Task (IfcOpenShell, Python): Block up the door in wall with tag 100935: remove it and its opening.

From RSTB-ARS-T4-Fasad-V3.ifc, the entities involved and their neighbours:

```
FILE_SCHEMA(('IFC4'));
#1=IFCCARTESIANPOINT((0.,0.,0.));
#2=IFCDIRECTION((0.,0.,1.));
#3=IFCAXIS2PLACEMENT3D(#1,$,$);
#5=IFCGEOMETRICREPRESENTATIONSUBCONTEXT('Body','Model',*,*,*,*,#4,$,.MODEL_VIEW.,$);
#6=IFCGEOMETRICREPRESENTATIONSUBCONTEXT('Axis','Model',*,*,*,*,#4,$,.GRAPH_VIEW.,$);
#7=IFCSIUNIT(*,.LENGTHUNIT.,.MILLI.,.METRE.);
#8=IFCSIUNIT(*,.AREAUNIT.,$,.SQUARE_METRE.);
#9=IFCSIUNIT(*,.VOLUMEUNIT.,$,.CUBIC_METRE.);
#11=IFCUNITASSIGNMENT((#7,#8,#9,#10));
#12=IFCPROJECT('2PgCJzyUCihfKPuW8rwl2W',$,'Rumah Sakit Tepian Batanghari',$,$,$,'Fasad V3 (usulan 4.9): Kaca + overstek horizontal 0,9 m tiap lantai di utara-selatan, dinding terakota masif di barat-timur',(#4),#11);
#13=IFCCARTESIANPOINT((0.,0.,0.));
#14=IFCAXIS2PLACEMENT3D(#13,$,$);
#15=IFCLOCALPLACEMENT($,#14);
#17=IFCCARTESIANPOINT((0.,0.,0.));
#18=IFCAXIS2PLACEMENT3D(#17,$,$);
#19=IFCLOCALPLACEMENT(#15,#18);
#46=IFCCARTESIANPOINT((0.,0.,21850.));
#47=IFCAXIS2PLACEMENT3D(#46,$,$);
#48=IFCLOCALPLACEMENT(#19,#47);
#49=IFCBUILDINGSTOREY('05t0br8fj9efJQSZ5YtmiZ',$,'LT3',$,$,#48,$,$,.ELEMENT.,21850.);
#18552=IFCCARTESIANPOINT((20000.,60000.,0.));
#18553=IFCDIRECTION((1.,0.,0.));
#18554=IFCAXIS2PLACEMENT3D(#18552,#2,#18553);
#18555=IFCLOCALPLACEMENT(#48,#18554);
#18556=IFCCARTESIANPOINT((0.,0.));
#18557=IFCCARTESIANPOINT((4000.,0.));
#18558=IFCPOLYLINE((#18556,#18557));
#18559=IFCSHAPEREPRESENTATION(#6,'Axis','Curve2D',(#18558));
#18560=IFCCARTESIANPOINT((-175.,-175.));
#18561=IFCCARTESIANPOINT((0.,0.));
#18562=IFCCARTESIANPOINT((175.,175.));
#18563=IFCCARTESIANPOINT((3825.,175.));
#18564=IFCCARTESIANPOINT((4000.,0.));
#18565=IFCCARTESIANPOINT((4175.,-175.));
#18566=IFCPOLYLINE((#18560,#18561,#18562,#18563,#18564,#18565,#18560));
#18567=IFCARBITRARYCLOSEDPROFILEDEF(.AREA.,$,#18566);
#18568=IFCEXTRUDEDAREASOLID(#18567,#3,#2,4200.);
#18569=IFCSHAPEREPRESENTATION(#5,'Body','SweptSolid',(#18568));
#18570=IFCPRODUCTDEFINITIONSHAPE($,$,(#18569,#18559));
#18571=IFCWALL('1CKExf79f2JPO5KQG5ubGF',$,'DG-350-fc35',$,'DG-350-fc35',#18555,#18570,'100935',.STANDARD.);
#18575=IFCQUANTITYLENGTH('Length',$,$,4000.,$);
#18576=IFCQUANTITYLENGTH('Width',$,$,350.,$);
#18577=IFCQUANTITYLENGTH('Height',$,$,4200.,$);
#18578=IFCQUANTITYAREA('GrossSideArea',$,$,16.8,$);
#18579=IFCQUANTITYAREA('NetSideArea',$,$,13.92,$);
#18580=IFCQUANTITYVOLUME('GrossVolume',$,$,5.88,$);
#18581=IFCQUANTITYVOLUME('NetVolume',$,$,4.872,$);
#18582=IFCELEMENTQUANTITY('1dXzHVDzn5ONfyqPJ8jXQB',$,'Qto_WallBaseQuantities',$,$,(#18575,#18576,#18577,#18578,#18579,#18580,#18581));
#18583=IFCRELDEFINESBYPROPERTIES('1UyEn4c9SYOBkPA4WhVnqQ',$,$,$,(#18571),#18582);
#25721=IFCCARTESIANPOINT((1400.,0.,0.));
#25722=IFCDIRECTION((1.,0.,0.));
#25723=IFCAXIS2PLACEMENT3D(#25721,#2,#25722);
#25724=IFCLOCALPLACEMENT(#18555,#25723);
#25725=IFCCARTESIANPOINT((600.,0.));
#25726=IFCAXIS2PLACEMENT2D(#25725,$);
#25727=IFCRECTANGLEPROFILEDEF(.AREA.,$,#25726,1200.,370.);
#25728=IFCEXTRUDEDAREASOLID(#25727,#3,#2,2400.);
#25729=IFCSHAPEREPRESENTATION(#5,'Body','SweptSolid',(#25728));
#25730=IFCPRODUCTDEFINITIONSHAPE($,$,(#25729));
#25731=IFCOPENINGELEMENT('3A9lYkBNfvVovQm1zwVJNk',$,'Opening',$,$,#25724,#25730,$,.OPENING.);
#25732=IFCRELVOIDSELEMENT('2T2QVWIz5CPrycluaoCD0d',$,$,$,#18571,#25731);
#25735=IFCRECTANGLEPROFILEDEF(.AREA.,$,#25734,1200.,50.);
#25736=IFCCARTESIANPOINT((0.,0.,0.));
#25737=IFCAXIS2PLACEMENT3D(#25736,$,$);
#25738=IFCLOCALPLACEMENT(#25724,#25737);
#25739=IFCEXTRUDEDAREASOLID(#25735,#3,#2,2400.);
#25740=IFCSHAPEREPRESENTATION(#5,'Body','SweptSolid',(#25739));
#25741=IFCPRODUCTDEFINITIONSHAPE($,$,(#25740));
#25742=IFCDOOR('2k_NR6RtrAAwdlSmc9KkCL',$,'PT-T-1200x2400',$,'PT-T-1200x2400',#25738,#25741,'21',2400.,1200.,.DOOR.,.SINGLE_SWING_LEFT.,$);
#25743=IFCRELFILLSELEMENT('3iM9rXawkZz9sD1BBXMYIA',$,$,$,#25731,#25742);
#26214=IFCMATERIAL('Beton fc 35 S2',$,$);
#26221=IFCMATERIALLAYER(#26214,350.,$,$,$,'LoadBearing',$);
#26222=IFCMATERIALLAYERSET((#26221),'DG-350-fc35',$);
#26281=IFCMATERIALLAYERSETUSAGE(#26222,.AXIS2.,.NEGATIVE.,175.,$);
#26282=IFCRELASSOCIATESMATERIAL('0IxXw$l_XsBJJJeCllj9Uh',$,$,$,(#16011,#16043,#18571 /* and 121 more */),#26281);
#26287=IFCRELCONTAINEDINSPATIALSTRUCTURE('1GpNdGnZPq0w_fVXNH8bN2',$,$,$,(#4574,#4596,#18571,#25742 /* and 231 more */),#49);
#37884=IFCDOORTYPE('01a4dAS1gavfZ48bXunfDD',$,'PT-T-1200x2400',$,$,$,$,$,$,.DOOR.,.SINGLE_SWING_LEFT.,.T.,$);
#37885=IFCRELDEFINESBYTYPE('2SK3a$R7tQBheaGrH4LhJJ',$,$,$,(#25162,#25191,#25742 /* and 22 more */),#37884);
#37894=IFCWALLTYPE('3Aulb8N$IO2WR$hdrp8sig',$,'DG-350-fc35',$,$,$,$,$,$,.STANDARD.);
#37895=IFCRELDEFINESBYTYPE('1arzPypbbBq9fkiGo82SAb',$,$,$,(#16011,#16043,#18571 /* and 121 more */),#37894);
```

```python
import ifcopenshell
import ifcopenshell.api.feature
import ifcopenshell.api.pset
import ifcopenshell.api.root
import ifcopenshell.geom
import ifcopenshell.util.element
import ifcopenshell.util.shape
import ifcopenshell.util.unit

model = ifcopenshell.open("RSTB-ARS-T4-Fasad-V3.ifc")
area_scale = ifcopenshell.util.unit.calculate_unit_scale(model, "AREAUNIT")
volume_scale = ifcopenshell.util.unit.calculate_unit_scale(model, "VOLUMEUNIT")
settings = ifcopenshell.geom.settings()


def volume(element):
    """Net volume in cubic metres, openings subtracted."""
    shape = ifcopenshell.geom.create_shape(settings, element)
    return ifcopenshell.util.shape.get_volume(shape.geometry)


door = model.by_id(25742)
opening = door.FillsVoids[0].RelatingOpeningElement
wall = opening.VoidsElements[0].RelatingBuildingElement
before = volume(wall)

ifcopenshell.api.root.remove_product(model, product=door)
ifcopenshell.api.feature.remove_feature(model, feature=opening)

after = volume(wall)
thickness = 0.35  # wall thickness in metres

# Update the wall's stored quantities.
qto = model.by_id(ifcopenshell.util.element.get_pset(wall, "Qto_WallBaseQuantities", should_inherit=False)["id"])
ifcopenshell.api.pset.edit_qto(model, qto=qto, properties={
    "NetSideArea": after / thickness / area_scale,
    "NetVolume": after / volume_scale,
})

print(f"wall volume {before:.3f} -> {after:.3f} m3")

model.write("RSTB-ARS-T4-Fasad-V3_updated.ifc")
```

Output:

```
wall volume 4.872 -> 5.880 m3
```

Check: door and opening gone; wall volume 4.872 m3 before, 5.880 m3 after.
